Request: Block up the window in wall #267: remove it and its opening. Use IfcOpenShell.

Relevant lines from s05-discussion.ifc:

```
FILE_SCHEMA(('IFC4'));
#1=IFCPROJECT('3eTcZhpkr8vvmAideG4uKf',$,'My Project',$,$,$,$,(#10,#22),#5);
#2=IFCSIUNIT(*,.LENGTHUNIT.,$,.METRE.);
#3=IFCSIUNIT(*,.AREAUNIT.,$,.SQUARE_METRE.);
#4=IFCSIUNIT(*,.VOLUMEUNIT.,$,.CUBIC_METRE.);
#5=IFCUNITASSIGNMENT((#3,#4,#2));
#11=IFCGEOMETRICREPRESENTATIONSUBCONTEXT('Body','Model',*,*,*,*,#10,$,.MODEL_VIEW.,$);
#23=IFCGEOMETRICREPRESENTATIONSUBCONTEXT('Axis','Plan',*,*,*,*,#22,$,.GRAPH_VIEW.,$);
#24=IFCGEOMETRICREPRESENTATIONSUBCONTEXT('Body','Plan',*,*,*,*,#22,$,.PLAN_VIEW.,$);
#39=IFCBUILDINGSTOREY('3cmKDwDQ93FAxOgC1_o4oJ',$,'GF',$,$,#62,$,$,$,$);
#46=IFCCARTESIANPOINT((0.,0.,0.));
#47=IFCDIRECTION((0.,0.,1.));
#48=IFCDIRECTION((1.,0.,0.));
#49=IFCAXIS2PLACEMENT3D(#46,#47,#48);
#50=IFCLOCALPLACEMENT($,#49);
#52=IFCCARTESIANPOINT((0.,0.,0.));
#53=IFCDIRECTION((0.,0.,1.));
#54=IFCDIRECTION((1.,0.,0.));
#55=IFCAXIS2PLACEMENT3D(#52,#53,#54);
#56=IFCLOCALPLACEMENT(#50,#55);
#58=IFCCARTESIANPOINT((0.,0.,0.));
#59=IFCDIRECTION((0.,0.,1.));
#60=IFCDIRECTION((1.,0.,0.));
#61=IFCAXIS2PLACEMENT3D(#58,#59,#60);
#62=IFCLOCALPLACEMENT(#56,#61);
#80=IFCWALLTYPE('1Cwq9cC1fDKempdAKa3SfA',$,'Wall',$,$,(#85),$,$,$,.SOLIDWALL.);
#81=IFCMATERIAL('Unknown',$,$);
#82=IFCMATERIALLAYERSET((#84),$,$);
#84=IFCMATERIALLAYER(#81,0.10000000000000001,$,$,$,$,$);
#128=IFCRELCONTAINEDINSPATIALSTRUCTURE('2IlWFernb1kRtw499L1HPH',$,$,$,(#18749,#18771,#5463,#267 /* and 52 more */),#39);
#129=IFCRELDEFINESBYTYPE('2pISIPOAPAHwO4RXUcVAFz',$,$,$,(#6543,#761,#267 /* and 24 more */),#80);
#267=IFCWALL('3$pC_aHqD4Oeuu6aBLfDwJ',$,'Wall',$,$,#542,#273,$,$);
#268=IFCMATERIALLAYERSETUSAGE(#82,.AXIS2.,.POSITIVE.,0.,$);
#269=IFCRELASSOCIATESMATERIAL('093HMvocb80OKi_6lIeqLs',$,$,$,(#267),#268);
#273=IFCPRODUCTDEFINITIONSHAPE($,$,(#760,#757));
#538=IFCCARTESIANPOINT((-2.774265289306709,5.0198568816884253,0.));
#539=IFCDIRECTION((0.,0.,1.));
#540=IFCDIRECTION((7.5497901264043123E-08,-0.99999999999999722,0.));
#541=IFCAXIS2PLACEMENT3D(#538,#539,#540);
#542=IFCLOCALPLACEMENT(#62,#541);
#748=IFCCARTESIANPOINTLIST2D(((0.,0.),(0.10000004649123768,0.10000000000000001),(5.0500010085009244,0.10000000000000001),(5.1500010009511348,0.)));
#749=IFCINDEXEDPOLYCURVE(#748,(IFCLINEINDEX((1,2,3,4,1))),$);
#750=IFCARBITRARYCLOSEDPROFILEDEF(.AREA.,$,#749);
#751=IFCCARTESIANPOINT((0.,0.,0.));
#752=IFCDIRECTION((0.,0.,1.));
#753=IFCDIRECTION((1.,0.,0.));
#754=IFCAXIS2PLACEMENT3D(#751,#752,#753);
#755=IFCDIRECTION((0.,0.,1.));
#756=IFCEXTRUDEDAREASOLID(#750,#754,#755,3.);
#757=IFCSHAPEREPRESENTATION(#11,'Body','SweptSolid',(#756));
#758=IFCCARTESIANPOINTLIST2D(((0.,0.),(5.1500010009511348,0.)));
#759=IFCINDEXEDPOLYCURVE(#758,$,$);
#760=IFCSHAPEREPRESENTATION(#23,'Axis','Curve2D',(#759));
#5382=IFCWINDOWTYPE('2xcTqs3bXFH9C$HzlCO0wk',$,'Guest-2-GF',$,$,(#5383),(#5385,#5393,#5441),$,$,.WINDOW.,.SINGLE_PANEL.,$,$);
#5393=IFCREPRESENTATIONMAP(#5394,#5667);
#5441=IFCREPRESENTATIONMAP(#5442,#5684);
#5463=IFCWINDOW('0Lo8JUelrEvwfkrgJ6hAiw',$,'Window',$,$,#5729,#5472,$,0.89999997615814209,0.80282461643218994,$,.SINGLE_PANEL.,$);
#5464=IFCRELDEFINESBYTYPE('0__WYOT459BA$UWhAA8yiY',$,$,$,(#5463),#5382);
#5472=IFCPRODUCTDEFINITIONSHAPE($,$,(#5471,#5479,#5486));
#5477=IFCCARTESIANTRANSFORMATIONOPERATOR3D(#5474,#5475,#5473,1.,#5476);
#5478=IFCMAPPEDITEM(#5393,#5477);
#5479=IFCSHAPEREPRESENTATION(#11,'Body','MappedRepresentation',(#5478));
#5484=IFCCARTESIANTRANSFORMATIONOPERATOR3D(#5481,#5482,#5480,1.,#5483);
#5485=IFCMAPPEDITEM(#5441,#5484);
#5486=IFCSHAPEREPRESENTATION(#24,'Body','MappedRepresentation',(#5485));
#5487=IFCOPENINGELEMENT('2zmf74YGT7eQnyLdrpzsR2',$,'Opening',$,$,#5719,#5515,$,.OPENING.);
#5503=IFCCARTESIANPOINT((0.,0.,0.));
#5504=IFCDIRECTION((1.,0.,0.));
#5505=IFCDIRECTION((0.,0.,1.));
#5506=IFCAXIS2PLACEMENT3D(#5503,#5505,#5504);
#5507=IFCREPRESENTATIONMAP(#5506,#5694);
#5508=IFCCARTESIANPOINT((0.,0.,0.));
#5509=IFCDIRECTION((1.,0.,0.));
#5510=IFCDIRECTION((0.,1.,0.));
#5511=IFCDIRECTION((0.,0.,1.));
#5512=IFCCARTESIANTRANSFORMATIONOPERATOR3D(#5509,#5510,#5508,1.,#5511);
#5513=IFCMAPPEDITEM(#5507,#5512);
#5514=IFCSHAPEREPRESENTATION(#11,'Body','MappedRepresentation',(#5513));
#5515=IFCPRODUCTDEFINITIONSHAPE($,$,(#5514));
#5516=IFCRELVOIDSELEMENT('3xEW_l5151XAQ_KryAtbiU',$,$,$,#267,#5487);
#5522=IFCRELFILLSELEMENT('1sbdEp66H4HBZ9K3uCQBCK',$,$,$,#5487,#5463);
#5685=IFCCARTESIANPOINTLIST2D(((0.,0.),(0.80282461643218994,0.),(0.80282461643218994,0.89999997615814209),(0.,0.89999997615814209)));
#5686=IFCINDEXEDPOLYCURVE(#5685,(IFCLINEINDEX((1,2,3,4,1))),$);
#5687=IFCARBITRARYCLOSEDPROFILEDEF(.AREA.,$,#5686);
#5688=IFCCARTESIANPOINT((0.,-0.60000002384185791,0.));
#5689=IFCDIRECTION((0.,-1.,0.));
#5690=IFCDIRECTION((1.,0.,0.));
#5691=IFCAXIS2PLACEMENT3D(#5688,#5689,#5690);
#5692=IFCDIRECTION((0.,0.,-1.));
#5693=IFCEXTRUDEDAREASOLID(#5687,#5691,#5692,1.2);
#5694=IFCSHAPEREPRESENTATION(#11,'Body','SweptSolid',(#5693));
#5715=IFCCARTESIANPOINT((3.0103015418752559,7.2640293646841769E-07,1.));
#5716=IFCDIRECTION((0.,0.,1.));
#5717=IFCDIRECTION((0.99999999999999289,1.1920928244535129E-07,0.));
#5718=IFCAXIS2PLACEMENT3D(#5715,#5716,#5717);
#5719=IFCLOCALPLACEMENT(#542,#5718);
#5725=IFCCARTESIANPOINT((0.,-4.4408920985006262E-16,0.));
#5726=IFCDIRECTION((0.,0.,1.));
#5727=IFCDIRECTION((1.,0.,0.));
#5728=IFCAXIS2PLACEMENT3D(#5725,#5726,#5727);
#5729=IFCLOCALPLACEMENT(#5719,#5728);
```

```python
import ifcopenshell
import ifcopenshell.api.feature
import ifcopenshell.api.root
import ifcopenshell.geom
import ifcopenshell.util.shape

model = ifcopenshell.open("s05-discussion.ifc")
settings = ifcopenshell.geom.settings()


def volume(element):
    """Net volume in cubic metres, openings subtracted."""
    shape = ifcopenshell.geom.create_shape(settings, element)
    return ifcopenshell.util.shape.get_volume(shape.geometry)


window = model.by_guid("0Lo8JUelrEvwfkrgJ6hAiw")
opening = window.FillsVoids[0].RelatingOpeningElement
wall = opening.VoidsElements[0].RelatingBuildingElement
before = volume(wall)

ifcopenshell.api.root.remove_product(model, product=window)
ifcopenshell.api.feature.remove_feature(model, feature=opening)

after = volume(wall)

print(f"wall volume {before:.3f} -> {after:.3f} m3")

model.write("s05-discussion_edited.ifc")
```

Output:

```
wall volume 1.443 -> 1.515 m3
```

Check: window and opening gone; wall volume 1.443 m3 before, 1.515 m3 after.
